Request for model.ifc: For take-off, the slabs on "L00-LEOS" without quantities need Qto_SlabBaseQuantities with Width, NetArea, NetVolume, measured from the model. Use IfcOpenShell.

First a look at what the model holds.

```python
import ifcopenshell
import ifcopenshell.util.element
import ifcopenshell.util.unit

model = ifcopenshell.open("model.ifc")
print(model.schema)
for unit_type in ("LENGTHUNIT", "AREAUNIT", "VOLUMEUNIT"):
    print(unit_type, ifcopenshell.util.unit.calculate_unit_scale(model, unit_type))
storey = next(s for s in model.by_type("IfcBuildingStorey") if s.Name == "L00-LEOS")
slabs = [e for e in ifcopenshell.util.element.get_decomposition(storey) if e.is_a("IfcSlab")]
for e in sorted(slabs, key=lambda e: e.id()):
    print(e.id(), e.is_a(), e.Name, list(ifcopenshell.util.element.get_psets(e, qtos_only=True)), sep=" | ")
```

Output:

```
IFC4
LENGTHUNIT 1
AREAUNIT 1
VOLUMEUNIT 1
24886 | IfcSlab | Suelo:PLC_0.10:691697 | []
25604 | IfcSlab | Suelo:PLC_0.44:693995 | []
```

```python
import ifcopenshell
import ifcopenshell.api.pset
import ifcopenshell.geom
import ifcopenshell.util.element
import ifcopenshell.util.shape
import ifcopenshell.util.unit

model = ifcopenshell.open("model.ifc")
unit_scale = ifcopenshell.util.unit.calculate_unit_scale(model)
area_scale = ifcopenshell.util.unit.calculate_unit_scale(model, "AREAUNIT")
volume_scale = ifcopenshell.util.unit.calculate_unit_scale(model, "VOLUMEUNIT")
settings = ifcopenshell.geom.settings()

storey = next(s for s in model.by_type("IfcBuildingStorey") if s.Name == "L00-LEOS")
slabs = [e for e in ifcopenshell.util.element.get_decomposition(storey) if e.is_a("IfcSlab")]

for e in sorted(slabs, key=lambda e: e.id()):
    if ifcopenshell.util.element.get_psets(e, qtos_only=True, should_inherit=False):
        continue
    # Geometry comes back in metres, in the element's own axes.
    shape = ifcopenshell.geom.create_shape(settings, e)
    values = {
        "Width": ifcopenshell.util.shape.get_z(shape.geometry) / unit_scale,
        "NetArea": ifcopenshell.util.shape.get_footprint_area(shape.geometry) / area_scale,
        "NetVolume": ifcopenshell.util.shape.get_volume(shape.geometry) / volume_scale,
    }
    qto = ifcopenshell.api.pset.add_qto(model, product=e, name="Qto_SlabBaseQuantities")
    ifcopenshell.api.pset.edit_qto(model, qto=qto, properties=values)
    print(e.id(), {k: round(v, 3) for k, v in values.items()})

model.write("model_updated.ifc")
```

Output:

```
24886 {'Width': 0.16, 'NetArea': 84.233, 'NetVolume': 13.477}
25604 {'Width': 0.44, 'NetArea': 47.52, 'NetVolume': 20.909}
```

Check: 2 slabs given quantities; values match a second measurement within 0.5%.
